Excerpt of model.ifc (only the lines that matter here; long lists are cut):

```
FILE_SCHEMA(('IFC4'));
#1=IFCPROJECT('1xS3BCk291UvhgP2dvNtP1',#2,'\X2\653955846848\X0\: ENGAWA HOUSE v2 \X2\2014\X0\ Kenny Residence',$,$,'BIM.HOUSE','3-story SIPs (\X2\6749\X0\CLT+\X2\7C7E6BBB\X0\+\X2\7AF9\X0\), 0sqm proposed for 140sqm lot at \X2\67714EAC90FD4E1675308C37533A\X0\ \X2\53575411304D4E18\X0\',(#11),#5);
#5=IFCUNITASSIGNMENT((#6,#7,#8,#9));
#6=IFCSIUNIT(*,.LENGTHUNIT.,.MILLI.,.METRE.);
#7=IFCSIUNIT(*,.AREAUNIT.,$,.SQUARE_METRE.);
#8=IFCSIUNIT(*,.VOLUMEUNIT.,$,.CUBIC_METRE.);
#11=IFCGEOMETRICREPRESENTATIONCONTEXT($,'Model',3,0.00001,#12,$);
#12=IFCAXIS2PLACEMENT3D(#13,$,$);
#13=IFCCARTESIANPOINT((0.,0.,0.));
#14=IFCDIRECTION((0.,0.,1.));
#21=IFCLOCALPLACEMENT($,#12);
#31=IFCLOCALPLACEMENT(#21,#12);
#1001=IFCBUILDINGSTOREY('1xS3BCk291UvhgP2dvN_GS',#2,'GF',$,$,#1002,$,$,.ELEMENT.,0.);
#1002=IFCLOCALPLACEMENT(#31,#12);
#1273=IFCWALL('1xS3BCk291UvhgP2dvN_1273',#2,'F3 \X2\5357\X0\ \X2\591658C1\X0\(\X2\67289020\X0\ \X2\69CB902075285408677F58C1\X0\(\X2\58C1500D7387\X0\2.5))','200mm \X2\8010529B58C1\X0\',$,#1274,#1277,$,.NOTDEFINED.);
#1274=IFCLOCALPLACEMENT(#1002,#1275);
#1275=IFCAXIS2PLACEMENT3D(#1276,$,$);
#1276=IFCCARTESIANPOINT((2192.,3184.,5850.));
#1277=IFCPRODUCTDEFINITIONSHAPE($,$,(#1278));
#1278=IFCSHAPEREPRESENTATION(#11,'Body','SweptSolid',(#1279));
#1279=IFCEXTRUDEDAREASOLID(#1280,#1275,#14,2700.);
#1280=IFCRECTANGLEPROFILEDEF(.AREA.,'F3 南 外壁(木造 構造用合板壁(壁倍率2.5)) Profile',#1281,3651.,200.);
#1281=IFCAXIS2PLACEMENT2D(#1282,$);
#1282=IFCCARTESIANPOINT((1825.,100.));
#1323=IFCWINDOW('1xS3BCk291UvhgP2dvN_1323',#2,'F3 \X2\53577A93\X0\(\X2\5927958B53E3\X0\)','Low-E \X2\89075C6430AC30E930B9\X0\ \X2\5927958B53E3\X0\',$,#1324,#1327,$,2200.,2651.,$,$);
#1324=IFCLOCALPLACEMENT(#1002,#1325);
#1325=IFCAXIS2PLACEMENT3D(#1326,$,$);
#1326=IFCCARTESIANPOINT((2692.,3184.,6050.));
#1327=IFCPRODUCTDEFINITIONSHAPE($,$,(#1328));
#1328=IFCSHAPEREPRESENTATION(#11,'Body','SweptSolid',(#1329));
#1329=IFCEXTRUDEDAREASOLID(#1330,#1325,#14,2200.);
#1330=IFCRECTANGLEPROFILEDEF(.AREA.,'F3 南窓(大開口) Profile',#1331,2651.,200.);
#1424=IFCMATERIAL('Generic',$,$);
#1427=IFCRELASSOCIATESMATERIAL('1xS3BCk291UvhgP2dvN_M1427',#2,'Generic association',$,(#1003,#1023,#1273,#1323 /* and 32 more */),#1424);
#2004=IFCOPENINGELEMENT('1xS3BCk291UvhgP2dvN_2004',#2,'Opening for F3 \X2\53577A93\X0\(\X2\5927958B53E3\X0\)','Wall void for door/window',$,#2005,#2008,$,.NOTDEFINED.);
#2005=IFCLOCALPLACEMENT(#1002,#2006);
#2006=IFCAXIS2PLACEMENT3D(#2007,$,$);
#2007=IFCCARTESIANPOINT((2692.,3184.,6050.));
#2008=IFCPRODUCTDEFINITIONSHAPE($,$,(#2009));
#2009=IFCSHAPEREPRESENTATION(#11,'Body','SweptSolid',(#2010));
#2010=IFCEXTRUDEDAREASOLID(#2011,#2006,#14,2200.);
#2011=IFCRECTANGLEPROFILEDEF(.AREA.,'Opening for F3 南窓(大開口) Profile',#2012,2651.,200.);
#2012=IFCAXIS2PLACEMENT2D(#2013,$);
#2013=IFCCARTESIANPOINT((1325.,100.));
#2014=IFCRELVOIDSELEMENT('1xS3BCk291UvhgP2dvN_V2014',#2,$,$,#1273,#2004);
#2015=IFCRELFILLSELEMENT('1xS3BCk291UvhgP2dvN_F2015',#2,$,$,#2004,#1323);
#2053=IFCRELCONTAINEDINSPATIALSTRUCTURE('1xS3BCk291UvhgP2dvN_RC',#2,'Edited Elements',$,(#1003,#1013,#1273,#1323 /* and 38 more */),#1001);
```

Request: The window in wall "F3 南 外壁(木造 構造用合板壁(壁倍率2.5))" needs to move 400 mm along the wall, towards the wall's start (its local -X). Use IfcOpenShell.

```python
import ifcopenshell
import ifcopenshell.api.geometry
import ifcopenshell.util.placement
import ifcopenshell.util.unit

model = ifcopenshell.open("model.ifc")
unit_scale = ifcopenshell.util.unit.calculate_unit_scale(model)

window = model.by_id(1323)
opening = window.FillsVoids[0].RelatingOpeningElement
wall = opening.VoidsElements[0].RelatingBuildingElement

wall_matrix = ifcopenshell.util.placement.get_local_placement(wall.ObjectPlacement)
shift = wall_matrix[:3, 0] * -0.4 / unit_scale
before = ifcopenshell.util.placement.get_local_placement(window.ObjectPlacement)[:3, 3].copy()

# The window is not placed relative to its opening, so move both.
for product in (opening, window):
    matrix = ifcopenshell.util.placement.get_local_placement(product.ObjectPlacement)
    matrix[:3, 3] += shift
    ifcopenshell.api.geometry.edit_object_placement(model, product=product, matrix=matrix, is_si=False)

after = ifcopenshell.util.placement.get_local_placement(window.ObjectPlacement)[:3, 3]
print("window moved by", (after - before).round(3) + 0.0)

model.write("model_v2.ifc")
```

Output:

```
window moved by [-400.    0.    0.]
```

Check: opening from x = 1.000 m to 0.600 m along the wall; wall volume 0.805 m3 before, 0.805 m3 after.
